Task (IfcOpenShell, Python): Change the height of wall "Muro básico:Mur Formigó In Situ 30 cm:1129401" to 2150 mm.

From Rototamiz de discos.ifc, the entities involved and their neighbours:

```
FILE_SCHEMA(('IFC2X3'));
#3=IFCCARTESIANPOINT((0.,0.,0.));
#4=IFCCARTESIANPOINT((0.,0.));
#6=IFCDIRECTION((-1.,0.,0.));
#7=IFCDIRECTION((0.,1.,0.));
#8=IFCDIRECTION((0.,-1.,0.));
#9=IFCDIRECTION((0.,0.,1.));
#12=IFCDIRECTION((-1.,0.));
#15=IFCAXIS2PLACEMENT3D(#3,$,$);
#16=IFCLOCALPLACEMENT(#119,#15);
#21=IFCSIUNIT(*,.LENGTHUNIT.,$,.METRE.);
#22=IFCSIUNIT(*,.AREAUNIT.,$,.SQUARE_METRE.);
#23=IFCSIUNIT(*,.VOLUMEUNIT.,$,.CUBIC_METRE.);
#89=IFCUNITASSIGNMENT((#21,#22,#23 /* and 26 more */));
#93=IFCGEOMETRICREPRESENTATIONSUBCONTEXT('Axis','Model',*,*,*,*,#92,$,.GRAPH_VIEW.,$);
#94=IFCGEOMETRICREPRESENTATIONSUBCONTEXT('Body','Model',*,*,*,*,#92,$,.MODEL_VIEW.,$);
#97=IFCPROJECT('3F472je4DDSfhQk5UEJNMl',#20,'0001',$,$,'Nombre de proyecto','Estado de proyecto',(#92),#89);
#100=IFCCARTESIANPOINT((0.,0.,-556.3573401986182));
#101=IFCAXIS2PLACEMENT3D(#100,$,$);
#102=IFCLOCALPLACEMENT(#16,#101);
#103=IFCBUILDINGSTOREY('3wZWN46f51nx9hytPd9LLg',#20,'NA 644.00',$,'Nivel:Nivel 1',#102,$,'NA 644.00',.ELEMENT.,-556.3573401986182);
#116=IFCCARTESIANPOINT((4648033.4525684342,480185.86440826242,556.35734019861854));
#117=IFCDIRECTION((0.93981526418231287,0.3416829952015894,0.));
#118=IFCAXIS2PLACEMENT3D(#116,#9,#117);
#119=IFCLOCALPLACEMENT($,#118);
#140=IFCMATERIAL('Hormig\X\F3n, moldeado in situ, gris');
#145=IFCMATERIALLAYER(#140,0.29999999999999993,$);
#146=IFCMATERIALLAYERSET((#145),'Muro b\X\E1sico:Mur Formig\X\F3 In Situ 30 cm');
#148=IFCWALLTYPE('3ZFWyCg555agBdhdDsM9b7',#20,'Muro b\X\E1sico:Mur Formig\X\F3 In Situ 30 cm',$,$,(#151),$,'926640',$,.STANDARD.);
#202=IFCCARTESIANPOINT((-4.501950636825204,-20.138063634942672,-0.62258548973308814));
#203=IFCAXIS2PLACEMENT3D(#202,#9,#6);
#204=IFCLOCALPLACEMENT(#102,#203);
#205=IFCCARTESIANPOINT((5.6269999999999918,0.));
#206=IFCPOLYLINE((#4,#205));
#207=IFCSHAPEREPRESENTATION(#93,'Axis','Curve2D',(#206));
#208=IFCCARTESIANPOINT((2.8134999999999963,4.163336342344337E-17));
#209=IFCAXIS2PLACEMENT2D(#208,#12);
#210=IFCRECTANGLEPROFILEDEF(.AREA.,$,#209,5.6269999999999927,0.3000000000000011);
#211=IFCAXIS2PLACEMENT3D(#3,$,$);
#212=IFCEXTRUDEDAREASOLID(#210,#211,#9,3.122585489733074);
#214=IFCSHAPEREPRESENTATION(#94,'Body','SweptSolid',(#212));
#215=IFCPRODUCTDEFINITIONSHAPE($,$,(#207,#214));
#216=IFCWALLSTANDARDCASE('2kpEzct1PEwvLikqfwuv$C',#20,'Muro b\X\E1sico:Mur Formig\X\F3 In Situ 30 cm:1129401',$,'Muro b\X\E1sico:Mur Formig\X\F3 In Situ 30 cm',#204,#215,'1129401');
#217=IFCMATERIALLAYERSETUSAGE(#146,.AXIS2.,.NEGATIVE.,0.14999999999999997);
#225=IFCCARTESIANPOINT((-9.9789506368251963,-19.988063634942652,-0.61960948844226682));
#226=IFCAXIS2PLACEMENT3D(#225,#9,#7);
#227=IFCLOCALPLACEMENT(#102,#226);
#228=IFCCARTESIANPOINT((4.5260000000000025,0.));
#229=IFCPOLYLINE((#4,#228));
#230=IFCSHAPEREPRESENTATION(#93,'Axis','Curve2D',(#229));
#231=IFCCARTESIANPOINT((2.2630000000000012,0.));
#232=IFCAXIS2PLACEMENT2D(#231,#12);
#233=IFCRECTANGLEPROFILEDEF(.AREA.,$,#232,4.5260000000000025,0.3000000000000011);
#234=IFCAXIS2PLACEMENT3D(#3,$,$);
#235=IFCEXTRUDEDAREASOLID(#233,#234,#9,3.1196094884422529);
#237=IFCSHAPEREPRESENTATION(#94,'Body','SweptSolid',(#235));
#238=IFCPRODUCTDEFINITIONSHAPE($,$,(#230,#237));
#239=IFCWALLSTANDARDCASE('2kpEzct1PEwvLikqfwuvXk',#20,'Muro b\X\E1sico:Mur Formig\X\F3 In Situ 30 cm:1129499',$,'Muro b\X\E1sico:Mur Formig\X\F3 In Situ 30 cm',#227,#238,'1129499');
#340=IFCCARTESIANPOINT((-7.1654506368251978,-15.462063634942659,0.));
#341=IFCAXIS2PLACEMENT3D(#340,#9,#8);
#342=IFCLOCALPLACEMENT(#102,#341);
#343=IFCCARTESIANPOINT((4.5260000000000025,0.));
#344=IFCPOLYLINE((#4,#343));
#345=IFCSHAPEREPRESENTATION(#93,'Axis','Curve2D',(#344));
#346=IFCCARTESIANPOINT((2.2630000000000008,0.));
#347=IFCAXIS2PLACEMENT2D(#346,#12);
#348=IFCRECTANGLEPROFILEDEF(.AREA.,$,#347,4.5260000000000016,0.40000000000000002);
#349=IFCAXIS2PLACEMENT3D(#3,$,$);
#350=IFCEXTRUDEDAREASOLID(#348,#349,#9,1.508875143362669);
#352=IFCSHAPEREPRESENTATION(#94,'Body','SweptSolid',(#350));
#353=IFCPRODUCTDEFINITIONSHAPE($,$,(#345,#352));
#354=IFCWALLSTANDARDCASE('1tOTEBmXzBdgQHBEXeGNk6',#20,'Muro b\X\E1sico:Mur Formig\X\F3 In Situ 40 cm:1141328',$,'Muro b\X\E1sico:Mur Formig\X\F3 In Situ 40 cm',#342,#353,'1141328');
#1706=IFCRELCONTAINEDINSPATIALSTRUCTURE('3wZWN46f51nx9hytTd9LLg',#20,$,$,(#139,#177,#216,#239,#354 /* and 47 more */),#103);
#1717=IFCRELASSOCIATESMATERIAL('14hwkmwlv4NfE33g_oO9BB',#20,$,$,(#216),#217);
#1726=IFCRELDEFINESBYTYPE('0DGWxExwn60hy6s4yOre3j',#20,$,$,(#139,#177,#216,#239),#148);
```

```python
import ifcopenshell
import ifcopenshell.geom
import ifcopenshell.util.representation
import ifcopenshell.util.shape
import ifcopenshell.util.unit

model = ifcopenshell.open("Rototamiz de discos.ifc")
unit_scale = ifcopenshell.util.unit.calculate_unit_scale(model)
settings = ifcopenshell.geom.settings()


def volume(element):
    """Net volume in cubic metres, openings subtracted."""
    shape = ifcopenshell.geom.create_shape(settings, element)
    return ifcopenshell.util.shape.get_volume(shape.geometry)


wall = model.by_guid("2kpEzct1PEwvLikqfwuv$C")
before = volume(wall)

body = ifcopenshell.util.representation.get_representation(wall, "Model", "Body")
solid = body.Items[0]
old_height = solid.Depth
solid.Depth = 2.15 / unit_scale
after = volume(wall)

print(f"height {old_height:g} -> {solid.Depth:g}, volume {before:.3f} -> {after:.3f} m3")

model.write("Rototamiz de discos-out.ifc")
```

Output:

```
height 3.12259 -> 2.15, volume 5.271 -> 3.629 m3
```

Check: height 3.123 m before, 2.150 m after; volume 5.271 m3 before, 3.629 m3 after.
